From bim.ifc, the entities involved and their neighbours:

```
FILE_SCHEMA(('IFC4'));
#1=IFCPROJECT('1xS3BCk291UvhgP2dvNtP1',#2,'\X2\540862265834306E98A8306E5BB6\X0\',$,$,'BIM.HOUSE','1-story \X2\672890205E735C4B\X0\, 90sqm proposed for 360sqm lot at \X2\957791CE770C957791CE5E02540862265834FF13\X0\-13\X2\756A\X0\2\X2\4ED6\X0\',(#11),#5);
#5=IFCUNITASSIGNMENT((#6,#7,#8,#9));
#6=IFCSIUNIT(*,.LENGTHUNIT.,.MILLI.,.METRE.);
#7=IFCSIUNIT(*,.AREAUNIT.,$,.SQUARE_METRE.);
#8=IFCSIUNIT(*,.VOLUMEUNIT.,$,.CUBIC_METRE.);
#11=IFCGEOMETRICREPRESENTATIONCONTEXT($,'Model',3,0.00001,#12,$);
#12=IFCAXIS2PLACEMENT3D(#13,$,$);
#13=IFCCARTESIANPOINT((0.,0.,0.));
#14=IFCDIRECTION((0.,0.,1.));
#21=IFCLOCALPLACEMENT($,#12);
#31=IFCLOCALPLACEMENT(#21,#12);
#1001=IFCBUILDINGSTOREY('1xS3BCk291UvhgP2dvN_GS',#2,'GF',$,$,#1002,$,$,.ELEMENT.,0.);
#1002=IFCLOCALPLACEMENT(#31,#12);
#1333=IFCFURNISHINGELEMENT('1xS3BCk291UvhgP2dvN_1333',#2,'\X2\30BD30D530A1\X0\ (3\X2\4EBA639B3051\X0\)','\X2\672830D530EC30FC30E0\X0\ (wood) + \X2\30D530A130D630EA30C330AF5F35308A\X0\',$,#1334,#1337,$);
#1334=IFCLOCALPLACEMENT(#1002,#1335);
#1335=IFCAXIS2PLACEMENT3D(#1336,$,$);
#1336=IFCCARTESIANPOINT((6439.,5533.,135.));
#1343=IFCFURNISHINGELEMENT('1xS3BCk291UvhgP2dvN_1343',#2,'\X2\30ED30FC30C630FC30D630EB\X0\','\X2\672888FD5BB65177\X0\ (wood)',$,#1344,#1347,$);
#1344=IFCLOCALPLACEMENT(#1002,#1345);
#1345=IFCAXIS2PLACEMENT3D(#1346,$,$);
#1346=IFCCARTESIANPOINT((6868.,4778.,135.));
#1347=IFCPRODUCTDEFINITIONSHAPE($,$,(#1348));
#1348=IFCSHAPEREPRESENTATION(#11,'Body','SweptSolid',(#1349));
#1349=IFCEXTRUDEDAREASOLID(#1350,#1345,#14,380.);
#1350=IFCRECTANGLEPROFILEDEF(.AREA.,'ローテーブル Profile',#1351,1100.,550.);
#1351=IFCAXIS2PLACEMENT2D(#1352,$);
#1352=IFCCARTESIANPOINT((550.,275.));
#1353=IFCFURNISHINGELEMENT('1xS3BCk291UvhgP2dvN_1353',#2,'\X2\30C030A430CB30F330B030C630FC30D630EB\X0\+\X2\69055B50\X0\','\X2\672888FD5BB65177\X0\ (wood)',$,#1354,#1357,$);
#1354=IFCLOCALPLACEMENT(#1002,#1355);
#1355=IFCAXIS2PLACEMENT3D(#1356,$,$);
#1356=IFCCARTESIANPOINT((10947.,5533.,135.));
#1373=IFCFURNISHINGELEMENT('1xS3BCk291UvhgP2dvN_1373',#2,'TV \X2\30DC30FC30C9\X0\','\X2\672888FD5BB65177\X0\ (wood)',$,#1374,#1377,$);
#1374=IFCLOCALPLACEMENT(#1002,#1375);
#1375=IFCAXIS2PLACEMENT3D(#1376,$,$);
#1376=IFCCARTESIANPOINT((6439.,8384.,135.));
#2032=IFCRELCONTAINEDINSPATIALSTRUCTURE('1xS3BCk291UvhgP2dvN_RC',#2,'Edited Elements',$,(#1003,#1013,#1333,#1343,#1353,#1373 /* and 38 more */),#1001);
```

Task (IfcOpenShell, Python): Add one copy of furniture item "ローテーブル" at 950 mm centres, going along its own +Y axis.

```python
import ifcopenshell
import ifcopenshell.api.geometry
import ifcopenshell.api.root
import ifcopenshell.util.element
import ifcopenshell.util.placement
import ifcopenshell.util.unit

model = ifcopenshell.open("bim.ifc")
unit_scale = ifcopenshell.util.unit.calculate_unit_scale(model)


def reuse_history(source, copy):
    """copy_class also copies each property set's owner history, people and application; keep the originals."""
    for rel in copy.IsDefinedBy:
        if rel.is_a("IfcRelDefinesByProperties") and (history := rel.RelatingPropertyDefinition.OwnerHistory):
            rel.RelatingPropertyDefinition.OwnerHistory = source.OwnerHistory
            ifcopenshell.util.element.remove_deep2(model, history)


source = model.by_id(1343)
base = ifcopenshell.util.placement.get_local_placement(source.ObjectPlacement)
step = base[:3, 1] * 0.95 / unit_scale

for i in range(1, 2):
    copy = ifcopenshell.api.root.copy_class(model, product=source)
    copy.Representation = ifcopenshell.util.element.copy_deep(
        model, source.Representation, exclude=["IfcGeometricRepresentationContext", "IfcRepresentationMap"]
    )
    reuse_history(source, copy)
    matrix = base.copy()
    matrix[:3, 3] += i * step
    print("added at", matrix[:3, 3].round(3) + 0.0)
    ifcopenshell.api.geometry.edit_object_placement(model, product=copy, matrix=matrix, is_si=False)

model.write("bim-out.ifc")
```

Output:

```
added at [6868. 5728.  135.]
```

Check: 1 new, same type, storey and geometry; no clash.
